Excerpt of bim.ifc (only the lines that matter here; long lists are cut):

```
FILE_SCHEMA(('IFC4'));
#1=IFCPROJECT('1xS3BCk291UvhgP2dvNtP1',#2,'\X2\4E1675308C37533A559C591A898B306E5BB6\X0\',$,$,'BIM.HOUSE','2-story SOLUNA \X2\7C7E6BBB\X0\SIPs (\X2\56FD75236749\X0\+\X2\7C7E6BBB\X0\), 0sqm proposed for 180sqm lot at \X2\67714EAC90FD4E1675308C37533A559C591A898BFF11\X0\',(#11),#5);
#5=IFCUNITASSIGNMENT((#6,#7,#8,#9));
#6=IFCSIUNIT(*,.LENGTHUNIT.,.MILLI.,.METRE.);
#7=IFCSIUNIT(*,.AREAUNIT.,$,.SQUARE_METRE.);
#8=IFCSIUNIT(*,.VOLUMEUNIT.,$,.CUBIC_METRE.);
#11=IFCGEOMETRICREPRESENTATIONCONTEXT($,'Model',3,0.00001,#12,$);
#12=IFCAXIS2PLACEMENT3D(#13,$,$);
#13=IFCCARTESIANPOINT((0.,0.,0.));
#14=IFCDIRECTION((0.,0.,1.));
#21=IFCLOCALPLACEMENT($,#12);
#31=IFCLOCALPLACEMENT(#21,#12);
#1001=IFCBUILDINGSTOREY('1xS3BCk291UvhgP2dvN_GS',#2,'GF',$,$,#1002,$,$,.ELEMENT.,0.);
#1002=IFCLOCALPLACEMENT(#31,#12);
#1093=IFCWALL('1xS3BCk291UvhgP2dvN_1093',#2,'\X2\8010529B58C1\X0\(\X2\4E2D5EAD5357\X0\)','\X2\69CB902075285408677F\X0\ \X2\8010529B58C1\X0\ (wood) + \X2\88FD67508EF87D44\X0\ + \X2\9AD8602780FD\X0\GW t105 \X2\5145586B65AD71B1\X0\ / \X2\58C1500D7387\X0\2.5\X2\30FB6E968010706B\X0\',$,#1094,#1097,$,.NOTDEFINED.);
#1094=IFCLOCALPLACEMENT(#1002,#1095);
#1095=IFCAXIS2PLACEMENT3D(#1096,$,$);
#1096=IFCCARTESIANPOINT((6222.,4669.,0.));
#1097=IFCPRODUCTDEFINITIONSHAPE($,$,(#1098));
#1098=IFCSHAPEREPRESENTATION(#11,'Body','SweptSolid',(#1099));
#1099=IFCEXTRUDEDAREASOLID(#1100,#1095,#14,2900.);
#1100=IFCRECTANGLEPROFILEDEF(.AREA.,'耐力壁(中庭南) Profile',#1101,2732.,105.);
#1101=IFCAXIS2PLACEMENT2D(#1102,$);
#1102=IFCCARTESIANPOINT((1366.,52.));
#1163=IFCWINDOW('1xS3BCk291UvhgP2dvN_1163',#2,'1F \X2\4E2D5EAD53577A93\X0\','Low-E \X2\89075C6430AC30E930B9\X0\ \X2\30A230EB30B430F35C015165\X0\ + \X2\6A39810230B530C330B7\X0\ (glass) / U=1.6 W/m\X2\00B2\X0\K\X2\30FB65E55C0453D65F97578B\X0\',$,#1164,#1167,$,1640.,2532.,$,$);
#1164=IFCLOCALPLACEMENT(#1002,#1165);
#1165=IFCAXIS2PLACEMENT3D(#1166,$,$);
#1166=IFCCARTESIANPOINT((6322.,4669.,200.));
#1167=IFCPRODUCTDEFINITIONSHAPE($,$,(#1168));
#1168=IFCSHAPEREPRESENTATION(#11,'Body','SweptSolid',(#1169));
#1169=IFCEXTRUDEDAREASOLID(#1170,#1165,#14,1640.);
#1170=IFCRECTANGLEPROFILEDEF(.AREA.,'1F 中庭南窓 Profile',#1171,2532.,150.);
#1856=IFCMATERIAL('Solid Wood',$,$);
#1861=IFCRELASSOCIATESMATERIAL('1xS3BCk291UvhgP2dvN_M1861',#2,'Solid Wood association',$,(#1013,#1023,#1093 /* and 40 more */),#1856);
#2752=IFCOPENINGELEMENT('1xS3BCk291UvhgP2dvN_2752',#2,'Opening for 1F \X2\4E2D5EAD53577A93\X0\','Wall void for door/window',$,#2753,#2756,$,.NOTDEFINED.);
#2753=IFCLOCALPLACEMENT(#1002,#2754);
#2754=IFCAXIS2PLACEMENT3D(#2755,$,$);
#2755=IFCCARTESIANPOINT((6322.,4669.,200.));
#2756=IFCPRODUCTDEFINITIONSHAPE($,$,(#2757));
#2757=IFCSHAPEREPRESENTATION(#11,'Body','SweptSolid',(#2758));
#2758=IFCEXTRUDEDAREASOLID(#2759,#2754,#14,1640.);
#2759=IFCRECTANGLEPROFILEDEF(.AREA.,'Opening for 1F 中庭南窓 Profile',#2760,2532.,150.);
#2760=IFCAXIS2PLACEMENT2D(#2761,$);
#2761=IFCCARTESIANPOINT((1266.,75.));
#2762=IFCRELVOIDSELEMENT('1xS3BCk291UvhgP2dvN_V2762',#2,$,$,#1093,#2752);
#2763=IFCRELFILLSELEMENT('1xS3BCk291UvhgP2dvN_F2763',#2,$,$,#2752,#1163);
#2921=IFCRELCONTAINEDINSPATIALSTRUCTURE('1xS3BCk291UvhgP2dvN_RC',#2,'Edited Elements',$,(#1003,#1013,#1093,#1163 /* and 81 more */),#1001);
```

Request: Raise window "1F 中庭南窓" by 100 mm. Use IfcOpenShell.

```python
import numpy as np
import ifcopenshell
import ifcopenshell.api.geometry
import ifcopenshell.util.placement
import ifcopenshell.util.unit

model = ifcopenshell.open("bim.ifc")
unit_scale = ifcopenshell.util.unit.calculate_unit_scale(model)

window = model.by_id(1163)
opening = window.FillsVoids[0].RelatingOpeningElement
dz = 100.0

shift = np.array([0.0, 0.0, dz])
# The window is not placed relative to its opening, so move both.
for product in (opening, window):
    matrix = ifcopenshell.util.placement.get_local_placement(product.ObjectPlacement)
    matrix[:3, 3] += shift
    ifcopenshell.api.geometry.edit_object_placement(model, product=product, matrix=matrix, is_si=False)

print(f"moved by {dz * unit_scale:+.3f} m")

model.write("bim_edited.ifc")
```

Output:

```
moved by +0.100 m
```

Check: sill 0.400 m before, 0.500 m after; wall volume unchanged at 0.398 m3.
